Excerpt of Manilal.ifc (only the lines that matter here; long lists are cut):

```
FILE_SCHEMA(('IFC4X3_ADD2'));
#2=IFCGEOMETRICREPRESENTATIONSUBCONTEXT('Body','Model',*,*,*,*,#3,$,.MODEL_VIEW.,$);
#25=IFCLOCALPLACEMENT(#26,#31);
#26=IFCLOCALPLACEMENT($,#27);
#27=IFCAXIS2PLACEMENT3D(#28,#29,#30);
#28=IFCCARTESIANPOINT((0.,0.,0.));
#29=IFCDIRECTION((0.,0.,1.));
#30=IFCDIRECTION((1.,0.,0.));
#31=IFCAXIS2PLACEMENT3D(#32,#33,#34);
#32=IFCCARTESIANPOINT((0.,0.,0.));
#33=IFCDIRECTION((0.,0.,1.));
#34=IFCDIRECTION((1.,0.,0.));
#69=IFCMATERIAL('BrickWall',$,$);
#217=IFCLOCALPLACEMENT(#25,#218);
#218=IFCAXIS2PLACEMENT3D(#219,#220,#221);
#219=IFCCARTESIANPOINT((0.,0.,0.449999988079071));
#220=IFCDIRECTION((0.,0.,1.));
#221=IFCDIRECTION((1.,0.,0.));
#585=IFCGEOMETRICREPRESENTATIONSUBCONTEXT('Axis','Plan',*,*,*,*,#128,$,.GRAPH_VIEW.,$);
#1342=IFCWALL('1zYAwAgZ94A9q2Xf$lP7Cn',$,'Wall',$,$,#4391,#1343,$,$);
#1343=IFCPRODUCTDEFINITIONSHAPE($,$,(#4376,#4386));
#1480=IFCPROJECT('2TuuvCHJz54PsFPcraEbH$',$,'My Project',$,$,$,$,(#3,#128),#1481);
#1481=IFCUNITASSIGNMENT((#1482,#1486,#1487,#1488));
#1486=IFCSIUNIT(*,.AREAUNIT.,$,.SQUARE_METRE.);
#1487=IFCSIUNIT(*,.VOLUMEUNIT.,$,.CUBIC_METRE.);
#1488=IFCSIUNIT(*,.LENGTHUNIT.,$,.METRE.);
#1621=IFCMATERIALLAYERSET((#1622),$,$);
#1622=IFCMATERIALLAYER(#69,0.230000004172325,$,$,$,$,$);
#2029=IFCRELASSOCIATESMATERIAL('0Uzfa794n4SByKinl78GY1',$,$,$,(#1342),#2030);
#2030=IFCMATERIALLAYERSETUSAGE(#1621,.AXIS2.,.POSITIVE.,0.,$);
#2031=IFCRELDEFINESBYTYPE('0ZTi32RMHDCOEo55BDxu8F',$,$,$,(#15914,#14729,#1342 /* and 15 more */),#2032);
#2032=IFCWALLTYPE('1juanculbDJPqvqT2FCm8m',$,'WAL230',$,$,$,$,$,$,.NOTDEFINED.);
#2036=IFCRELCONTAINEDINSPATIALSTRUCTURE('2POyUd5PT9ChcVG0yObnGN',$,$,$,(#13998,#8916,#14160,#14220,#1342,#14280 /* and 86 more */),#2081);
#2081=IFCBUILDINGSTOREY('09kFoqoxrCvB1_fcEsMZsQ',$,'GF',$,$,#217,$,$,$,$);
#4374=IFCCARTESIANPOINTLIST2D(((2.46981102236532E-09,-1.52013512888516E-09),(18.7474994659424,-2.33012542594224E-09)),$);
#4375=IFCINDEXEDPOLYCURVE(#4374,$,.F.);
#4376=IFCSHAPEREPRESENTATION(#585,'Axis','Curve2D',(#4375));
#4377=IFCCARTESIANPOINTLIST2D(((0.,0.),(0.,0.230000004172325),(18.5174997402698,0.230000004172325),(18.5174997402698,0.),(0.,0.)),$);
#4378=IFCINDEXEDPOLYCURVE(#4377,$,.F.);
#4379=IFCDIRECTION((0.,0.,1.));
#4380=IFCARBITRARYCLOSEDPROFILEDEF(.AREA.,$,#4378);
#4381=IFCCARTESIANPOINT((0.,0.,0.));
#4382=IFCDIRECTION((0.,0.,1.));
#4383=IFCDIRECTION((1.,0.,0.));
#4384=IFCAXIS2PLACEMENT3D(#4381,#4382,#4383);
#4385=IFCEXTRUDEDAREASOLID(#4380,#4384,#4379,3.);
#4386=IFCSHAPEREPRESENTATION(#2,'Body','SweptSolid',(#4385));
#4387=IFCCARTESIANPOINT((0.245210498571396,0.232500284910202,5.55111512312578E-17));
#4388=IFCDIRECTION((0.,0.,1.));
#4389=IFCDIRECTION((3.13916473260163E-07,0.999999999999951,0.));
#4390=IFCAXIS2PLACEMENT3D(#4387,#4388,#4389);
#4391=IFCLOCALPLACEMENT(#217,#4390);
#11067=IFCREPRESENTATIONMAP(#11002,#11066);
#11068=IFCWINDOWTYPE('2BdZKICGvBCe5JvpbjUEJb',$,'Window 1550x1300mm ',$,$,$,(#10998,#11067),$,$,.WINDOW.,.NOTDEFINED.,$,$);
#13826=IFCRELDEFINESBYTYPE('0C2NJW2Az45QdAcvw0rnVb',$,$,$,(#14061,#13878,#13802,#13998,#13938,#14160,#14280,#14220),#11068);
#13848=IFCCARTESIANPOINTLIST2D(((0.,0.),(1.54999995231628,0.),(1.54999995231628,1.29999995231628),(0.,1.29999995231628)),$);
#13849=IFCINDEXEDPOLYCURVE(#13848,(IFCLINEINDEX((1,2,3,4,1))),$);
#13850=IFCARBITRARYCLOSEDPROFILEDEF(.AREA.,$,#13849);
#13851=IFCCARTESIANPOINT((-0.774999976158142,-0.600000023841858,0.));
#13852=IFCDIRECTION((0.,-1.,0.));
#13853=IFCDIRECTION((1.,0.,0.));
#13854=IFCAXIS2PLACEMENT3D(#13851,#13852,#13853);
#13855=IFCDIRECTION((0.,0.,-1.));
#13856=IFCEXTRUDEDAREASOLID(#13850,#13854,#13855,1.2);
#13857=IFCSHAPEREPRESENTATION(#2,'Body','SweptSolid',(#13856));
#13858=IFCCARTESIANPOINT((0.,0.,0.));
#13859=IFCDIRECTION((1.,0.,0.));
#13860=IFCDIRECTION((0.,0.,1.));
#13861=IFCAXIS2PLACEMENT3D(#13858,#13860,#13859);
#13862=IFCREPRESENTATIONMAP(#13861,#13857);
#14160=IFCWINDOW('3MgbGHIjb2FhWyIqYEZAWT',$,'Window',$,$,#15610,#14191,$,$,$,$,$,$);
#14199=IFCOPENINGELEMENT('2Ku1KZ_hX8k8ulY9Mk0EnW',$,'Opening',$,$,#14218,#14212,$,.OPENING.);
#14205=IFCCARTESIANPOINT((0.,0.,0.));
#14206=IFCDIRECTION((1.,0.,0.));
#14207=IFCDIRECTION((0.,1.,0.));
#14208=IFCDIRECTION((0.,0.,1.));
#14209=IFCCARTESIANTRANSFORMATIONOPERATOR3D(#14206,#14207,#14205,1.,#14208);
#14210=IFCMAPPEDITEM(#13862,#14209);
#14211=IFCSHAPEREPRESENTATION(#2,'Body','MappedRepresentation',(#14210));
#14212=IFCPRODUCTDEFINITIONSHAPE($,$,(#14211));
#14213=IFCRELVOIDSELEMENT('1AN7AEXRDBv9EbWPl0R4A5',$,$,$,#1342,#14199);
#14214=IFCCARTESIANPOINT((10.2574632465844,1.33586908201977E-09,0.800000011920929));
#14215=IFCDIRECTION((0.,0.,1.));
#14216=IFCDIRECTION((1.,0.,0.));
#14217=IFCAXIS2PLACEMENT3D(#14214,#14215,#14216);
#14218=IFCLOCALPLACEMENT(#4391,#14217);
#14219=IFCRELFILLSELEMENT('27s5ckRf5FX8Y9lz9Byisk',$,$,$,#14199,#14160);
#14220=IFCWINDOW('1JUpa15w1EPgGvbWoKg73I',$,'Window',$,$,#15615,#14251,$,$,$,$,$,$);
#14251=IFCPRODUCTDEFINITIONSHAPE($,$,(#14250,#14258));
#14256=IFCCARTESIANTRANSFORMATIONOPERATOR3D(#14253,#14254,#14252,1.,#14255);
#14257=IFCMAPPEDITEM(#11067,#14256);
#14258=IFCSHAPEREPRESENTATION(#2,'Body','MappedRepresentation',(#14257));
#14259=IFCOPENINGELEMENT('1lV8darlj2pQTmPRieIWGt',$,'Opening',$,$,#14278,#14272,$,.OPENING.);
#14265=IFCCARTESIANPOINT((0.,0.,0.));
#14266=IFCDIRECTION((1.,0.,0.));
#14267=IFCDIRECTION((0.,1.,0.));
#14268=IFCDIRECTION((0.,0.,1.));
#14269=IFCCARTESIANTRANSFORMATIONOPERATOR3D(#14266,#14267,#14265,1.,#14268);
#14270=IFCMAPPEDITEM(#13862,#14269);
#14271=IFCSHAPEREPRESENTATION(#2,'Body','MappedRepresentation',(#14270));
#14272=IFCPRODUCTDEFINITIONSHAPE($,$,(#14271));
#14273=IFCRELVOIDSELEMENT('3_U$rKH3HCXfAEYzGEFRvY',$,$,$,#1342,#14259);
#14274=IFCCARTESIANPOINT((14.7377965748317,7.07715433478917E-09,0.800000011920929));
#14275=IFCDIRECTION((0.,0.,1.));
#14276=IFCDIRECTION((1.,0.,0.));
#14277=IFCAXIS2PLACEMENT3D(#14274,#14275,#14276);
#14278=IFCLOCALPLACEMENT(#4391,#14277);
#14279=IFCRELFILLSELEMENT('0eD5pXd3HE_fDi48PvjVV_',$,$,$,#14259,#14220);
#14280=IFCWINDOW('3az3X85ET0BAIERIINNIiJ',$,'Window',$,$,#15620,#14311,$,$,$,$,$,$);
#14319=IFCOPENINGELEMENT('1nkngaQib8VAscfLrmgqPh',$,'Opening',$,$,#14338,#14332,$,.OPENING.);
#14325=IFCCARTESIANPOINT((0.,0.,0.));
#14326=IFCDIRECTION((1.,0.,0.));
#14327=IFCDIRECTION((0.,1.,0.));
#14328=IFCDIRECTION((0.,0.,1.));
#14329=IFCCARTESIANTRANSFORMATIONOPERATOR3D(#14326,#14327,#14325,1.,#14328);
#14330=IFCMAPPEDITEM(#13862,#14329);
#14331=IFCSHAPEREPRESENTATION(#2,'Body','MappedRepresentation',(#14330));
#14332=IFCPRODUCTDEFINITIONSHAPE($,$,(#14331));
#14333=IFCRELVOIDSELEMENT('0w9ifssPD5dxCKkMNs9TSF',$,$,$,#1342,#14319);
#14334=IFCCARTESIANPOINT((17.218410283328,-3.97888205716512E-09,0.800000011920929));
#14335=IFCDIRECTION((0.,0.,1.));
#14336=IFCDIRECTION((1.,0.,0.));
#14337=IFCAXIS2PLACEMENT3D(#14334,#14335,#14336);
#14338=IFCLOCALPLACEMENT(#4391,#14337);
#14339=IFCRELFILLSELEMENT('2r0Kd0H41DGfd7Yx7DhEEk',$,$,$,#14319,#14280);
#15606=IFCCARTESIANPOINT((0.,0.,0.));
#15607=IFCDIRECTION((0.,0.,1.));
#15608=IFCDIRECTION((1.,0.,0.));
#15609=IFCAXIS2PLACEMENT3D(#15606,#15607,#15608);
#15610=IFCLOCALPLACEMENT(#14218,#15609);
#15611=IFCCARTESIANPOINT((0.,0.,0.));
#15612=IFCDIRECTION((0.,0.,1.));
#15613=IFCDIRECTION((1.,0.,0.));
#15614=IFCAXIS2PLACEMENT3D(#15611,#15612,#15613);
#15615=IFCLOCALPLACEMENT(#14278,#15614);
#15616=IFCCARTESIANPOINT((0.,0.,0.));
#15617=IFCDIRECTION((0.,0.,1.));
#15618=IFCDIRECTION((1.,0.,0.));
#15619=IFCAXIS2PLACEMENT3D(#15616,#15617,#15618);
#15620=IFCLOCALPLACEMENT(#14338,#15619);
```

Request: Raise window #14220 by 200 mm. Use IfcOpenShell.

```python
import numpy as np
import ifcopenshell
import ifcopenshell.api.geometry
import ifcopenshell.util.placement
import ifcopenshell.util.unit

model = ifcopenshell.open("Manilal.ifc")
unit_scale = ifcopenshell.util.unit.calculate_unit_scale(model)

window = model.by_id(14220)
opening = window.FillsVoids[0].RelatingOpeningElement
dz = 0.2 / unit_scale

shift = np.array([0.0, 0.0, dz])
# The window is placed relative to its opening, so it follows when the opening moves.
matrix = ifcopenshell.util.placement.get_local_placement(opening.ObjectPlacement)
matrix[:3, 3] += shift
ifcopenshell.api.geometry.edit_object_placement(
    model, product=opening, matrix=matrix, is_si=False, should_transform_children=True
)

print(f"moved by {dz * unit_scale:+.3f} m")

model.write("Manilal_rev.ifc")
```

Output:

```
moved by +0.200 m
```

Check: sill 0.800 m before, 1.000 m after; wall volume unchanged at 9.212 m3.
